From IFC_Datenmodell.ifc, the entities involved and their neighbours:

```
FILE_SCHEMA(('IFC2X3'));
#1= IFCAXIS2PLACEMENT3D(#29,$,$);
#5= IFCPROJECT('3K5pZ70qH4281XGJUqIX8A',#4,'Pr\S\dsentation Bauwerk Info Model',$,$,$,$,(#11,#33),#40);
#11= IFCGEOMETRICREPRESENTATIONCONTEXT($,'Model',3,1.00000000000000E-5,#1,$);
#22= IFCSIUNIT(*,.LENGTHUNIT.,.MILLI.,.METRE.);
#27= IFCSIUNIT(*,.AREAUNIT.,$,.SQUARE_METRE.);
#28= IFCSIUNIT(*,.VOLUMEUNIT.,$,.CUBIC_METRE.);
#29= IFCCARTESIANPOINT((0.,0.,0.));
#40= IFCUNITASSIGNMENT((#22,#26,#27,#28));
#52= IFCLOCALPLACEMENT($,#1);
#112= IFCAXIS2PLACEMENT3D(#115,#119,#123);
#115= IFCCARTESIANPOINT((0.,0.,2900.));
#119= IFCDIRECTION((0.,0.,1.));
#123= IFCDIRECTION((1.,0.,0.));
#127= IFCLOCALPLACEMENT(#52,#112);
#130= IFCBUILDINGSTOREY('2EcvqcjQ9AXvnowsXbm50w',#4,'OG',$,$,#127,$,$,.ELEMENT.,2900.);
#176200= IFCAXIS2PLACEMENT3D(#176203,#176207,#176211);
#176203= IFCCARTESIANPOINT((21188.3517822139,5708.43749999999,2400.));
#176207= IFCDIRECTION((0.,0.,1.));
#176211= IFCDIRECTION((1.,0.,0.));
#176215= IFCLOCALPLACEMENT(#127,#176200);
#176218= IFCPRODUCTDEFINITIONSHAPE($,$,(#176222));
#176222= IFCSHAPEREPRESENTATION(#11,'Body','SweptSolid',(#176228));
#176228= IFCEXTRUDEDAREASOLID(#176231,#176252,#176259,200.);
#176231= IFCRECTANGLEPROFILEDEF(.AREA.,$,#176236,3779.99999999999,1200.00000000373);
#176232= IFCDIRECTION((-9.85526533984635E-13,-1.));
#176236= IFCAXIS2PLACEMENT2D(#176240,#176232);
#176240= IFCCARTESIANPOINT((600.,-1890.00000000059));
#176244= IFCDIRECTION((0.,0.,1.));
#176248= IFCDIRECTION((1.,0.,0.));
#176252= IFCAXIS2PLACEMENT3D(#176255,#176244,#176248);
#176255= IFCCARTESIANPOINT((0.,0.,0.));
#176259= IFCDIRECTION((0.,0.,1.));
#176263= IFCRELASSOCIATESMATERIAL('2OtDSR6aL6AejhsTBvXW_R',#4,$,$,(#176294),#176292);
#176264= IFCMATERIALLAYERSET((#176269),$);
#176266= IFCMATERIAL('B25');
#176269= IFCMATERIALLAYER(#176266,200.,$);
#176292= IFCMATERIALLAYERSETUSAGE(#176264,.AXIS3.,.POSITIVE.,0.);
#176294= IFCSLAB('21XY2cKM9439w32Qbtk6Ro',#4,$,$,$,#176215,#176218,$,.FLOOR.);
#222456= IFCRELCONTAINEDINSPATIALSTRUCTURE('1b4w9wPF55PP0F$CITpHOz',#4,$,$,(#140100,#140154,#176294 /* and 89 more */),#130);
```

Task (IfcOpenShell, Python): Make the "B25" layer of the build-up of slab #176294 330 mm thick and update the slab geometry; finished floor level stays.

```python
import ifcopenshell
import ifcopenshell.util.element
import ifcopenshell.util.unit

model = ifcopenshell.open("IFC_Datenmodell.ifc")
unit_scale = ifcopenshell.util.unit.calculate_unit_scale(model)

layer_set = model.by_id(176264)
layer = next(l for l in layer_set.MaterialLayers if l.Material and l.Material.Name == "B25")
change = 0.33 / unit_scale - layer.LayerThickness
layer.LayerThickness += change

# Geometry does not follow the layer set by itself.
slabs = [e for e in ifcopenshell.util.element.get_elements_by_material(model, layer_set) if e.is_a("IfcSlab")]
for slab in sorted(slabs, key=lambda e: e.id()):
    body = next(r for r in slab.Representation.Representations if r.RepresentationIdentifier == "Body")
    solid = body.Items[0]
    old_depth = solid.Depth
    solid.Depth += change
    # Extruded upwards: lower the start of the extrusion so the top stays.
    x, y, z = solid.Position.Location.Coordinates
    solid.Position.Location = model.createIfcCartesianPoint((x, y, z - change))
    print(slab.id(), f"{old_depth:g} -> {solid.Depth:g}")

# The layers are counted up from the underside, which has moved.
for usage in {ifcopenshell.util.element.get_material(slab) for slab in slabs}:
    usage.OffsetFromReferenceLine -= change

model.write("IFC_Datenmodell-out.ifc")
```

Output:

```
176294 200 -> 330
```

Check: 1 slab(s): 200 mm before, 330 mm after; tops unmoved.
